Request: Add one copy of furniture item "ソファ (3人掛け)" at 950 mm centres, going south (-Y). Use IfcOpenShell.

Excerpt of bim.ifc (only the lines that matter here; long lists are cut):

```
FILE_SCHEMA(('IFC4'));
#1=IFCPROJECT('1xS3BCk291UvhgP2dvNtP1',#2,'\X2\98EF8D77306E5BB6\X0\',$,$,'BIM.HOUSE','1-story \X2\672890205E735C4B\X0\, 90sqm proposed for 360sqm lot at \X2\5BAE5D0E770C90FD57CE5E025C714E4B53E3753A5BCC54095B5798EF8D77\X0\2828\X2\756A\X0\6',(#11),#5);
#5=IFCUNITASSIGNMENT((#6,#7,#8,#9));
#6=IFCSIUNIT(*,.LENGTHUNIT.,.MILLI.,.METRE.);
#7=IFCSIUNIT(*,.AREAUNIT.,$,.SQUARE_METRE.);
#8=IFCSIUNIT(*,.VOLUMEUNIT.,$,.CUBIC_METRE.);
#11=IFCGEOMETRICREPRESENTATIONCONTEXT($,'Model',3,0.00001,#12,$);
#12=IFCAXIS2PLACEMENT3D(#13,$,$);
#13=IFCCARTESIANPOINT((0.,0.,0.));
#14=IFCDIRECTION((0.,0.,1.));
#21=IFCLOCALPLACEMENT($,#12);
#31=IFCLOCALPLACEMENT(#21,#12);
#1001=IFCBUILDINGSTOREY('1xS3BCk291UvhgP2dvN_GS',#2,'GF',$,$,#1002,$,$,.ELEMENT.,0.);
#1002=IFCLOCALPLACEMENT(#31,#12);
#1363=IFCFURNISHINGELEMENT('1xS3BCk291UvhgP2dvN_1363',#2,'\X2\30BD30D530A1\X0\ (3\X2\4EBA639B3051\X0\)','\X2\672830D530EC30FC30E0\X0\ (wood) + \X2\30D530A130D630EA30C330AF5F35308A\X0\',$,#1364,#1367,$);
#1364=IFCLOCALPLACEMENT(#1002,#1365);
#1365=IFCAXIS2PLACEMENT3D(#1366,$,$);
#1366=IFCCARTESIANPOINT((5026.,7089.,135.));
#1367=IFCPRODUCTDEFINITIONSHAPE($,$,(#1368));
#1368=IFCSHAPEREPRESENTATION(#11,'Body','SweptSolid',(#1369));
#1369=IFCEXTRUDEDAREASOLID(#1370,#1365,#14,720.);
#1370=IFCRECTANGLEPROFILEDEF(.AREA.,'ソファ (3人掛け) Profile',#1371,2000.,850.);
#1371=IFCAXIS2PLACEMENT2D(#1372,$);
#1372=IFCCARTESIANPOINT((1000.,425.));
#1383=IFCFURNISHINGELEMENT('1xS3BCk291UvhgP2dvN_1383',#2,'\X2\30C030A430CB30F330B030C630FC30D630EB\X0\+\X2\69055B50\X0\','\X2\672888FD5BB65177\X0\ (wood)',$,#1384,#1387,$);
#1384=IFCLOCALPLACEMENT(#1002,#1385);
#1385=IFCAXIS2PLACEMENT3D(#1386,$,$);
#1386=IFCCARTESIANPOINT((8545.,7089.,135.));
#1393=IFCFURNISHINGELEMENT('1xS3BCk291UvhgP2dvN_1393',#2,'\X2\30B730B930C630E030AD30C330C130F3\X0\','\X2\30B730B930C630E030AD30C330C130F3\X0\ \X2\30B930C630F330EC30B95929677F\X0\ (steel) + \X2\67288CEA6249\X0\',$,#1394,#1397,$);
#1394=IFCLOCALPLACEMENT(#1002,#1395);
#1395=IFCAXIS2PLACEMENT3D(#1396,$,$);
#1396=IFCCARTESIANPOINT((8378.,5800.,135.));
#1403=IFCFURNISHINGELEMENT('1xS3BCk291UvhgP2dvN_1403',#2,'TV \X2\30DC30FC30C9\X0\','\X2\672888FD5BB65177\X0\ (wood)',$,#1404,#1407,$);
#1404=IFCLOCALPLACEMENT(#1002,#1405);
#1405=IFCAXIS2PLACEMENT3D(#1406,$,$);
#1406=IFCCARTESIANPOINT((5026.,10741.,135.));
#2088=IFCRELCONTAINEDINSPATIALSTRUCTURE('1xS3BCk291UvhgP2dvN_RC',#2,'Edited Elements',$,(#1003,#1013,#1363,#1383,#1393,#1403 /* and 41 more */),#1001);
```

```python
import numpy as np
import ifcopenshell
import ifcopenshell.api.geometry
import ifcopenshell.api.root
import ifcopenshell.util.element
import ifcopenshell.util.placement
import ifcopenshell.util.unit

model = ifcopenshell.open("bim.ifc")
unit_scale = ifcopenshell.util.unit.calculate_unit_scale(model)


def reuse_history(source, copy):
    """copy_class also copies each property set's owner history, people and application; keep the originals."""
    for rel in copy.IsDefinedBy:
        if rel.is_a("IfcRelDefinesByProperties") and (history := rel.RelatingPropertyDefinition.OwnerHistory):
            rel.RelatingPropertyDefinition.OwnerHistory = source.OwnerHistory
            ifcopenshell.util.element.remove_deep2(model, history)


source = model.by_guid("1xS3BCk291UvhgP2dvN_1363")
base = ifcopenshell.util.placement.get_local_placement(source.ObjectPlacement)
step = np.array([0.0, -1.0, 0.0]) * 0.95 / unit_scale

for i in range(1, 2):
    copy = ifcopenshell.api.root.copy_class(model, product=source)
    copy.Representation = ifcopenshell.util.element.copy_deep(
        model, source.Representation, exclude=["IfcGeometricRepresentationContext", "IfcRepresentationMap"]
    )
    reuse_history(source, copy)
    matrix = base.copy()
    matrix[:3, 3] += i * step
    print("added at", matrix[:3, 3].round(3) + 0.0)
    ifcopenshell.api.geometry.edit_object_placement(model, product=copy, matrix=matrix, is_si=False)

model.write("bim_updated.ifc")
```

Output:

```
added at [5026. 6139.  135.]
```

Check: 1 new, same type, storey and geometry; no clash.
